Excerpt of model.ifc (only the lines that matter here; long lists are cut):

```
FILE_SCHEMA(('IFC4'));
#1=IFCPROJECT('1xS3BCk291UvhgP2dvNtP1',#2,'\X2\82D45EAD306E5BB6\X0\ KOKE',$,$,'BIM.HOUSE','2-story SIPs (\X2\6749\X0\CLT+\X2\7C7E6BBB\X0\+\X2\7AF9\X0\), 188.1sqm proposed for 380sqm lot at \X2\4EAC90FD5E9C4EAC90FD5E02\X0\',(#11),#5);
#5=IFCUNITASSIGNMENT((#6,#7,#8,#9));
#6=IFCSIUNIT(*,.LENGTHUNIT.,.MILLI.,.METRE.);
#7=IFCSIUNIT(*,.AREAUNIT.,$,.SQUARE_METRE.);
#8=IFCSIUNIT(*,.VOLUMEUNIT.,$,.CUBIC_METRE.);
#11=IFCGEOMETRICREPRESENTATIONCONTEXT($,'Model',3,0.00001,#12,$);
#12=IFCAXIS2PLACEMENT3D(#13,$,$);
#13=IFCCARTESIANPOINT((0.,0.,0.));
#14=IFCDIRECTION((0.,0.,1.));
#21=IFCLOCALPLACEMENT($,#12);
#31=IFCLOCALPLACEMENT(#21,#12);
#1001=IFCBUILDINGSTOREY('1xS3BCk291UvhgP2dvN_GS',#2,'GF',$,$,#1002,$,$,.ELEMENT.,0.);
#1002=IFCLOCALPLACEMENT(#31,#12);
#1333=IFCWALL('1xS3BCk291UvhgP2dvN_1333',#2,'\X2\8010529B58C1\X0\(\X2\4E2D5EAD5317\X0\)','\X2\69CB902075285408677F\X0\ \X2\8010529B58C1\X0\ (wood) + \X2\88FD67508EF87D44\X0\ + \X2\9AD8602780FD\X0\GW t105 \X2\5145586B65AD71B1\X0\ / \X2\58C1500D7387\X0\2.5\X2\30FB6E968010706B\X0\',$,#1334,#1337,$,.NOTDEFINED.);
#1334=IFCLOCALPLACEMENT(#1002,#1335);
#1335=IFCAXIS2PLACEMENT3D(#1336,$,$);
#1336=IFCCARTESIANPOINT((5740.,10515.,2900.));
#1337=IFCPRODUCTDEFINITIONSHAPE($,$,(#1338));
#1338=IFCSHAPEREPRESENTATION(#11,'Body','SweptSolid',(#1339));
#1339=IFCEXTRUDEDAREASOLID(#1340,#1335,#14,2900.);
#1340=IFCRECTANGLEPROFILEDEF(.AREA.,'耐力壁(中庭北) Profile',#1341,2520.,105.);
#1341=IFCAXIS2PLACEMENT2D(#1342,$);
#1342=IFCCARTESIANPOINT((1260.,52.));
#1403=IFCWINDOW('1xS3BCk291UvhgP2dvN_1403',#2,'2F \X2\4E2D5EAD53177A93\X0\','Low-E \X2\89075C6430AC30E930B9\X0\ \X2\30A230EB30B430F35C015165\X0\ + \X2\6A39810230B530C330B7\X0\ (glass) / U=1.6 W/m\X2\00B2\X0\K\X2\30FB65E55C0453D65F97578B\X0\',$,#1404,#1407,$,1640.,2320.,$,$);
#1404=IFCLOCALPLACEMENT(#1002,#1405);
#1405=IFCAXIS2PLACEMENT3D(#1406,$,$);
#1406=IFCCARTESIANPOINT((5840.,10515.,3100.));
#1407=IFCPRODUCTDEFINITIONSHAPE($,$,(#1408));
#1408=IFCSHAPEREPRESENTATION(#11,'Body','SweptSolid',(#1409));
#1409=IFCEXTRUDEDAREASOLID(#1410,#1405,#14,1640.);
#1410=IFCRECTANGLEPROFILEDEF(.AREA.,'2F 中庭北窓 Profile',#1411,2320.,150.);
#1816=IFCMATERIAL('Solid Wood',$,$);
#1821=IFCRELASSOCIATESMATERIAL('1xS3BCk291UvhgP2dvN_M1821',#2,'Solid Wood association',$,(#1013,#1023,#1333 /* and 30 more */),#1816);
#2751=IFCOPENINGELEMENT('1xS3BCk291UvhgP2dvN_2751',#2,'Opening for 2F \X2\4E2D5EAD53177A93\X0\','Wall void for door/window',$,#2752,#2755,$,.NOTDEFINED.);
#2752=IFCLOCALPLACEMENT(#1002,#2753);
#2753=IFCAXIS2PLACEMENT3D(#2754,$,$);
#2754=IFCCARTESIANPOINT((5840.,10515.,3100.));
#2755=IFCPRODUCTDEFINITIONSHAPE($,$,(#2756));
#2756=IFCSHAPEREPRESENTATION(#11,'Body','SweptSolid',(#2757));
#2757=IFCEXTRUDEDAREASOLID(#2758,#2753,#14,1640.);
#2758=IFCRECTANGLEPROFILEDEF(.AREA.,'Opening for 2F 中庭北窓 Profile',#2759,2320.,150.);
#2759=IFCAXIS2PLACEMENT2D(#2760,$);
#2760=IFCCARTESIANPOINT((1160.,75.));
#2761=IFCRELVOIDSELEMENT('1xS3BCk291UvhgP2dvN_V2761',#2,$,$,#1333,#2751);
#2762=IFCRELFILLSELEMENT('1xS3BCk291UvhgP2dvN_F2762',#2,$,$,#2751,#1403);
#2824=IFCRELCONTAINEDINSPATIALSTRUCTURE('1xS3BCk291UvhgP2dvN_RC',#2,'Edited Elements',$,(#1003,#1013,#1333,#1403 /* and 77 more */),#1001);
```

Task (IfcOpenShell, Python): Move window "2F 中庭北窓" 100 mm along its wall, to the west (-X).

```python
import ifcopenshell
import ifcopenshell.api.geometry
import ifcopenshell.util.placement

model = ifcopenshell.open("model.ifc")

window = model.by_id(1403)
opening = window.FillsVoids[0].RelatingOpeningElement
wall = opening.VoidsElements[0].RelatingBuildingElement

wall_matrix = ifcopenshell.util.placement.get_local_placement(wall.ObjectPlacement)
shift = wall_matrix[:3, 0] * -100.0
before = ifcopenshell.util.placement.get_local_placement(window.ObjectPlacement)[:3, 3].copy()

# The window is not placed relative to its opening, so move both.
for product in (opening, window):
    matrix = ifcopenshell.util.placement.get_local_placement(product.ObjectPlacement)
    matrix[:3, 3] += shift
    ifcopenshell.api.geometry.edit_object_placement(model, product=product, matrix=matrix, is_si=False)

after = ifcopenshell.util.placement.get_local_placement(window.ObjectPlacement)[:3, 3]
print("window moved by", (after - before).round(3) + 0.0)

model.write("model_rev.ifc")
```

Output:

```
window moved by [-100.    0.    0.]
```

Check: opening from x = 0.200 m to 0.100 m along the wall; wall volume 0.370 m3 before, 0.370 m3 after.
